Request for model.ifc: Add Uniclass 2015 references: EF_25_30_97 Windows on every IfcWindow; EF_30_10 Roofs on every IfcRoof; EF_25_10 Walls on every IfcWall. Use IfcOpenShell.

First a look at what the model holds.

```python
import ifcopenshell

model = ifcopenshell.open("model.ifc")
print(model.schema)
print("classifications:", [c.Name for c in model.by_type("IfcClassification")])
for ifc_class in ("IfcDoor", "IfcRoof", "IfcStair", "IfcWall", "IfcWindow"):
    print(ifc_class, len(model.by_type(ifc_class)))
```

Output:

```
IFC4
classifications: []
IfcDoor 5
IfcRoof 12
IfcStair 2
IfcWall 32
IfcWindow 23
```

```python
import ifcopenshell
import ifcopenshell.api.classification

model = ifcopenshell.open("model.ifc")

system = ifcopenshell.api.classification.add_classification(model, classification="Uniclass 2015")

codes = {
    "IfcWindow": ("EF_25_30_97", "Windows"),
    "IfcRoof": ("EF_30_10", "Roofs"),
    "IfcWall": ("EF_25_10", "Walls"),
}
for ifc_class, (code, name) in codes.items():
    products = model.by_type(ifc_class)
    ifcopenshell.api.classification.add_reference(
        model, products=products, classification=system, identification=code, name=name
    )
    print(code, len(products))

model.write("model_v2.ifc")
```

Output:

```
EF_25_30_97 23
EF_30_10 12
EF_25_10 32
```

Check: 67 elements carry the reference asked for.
